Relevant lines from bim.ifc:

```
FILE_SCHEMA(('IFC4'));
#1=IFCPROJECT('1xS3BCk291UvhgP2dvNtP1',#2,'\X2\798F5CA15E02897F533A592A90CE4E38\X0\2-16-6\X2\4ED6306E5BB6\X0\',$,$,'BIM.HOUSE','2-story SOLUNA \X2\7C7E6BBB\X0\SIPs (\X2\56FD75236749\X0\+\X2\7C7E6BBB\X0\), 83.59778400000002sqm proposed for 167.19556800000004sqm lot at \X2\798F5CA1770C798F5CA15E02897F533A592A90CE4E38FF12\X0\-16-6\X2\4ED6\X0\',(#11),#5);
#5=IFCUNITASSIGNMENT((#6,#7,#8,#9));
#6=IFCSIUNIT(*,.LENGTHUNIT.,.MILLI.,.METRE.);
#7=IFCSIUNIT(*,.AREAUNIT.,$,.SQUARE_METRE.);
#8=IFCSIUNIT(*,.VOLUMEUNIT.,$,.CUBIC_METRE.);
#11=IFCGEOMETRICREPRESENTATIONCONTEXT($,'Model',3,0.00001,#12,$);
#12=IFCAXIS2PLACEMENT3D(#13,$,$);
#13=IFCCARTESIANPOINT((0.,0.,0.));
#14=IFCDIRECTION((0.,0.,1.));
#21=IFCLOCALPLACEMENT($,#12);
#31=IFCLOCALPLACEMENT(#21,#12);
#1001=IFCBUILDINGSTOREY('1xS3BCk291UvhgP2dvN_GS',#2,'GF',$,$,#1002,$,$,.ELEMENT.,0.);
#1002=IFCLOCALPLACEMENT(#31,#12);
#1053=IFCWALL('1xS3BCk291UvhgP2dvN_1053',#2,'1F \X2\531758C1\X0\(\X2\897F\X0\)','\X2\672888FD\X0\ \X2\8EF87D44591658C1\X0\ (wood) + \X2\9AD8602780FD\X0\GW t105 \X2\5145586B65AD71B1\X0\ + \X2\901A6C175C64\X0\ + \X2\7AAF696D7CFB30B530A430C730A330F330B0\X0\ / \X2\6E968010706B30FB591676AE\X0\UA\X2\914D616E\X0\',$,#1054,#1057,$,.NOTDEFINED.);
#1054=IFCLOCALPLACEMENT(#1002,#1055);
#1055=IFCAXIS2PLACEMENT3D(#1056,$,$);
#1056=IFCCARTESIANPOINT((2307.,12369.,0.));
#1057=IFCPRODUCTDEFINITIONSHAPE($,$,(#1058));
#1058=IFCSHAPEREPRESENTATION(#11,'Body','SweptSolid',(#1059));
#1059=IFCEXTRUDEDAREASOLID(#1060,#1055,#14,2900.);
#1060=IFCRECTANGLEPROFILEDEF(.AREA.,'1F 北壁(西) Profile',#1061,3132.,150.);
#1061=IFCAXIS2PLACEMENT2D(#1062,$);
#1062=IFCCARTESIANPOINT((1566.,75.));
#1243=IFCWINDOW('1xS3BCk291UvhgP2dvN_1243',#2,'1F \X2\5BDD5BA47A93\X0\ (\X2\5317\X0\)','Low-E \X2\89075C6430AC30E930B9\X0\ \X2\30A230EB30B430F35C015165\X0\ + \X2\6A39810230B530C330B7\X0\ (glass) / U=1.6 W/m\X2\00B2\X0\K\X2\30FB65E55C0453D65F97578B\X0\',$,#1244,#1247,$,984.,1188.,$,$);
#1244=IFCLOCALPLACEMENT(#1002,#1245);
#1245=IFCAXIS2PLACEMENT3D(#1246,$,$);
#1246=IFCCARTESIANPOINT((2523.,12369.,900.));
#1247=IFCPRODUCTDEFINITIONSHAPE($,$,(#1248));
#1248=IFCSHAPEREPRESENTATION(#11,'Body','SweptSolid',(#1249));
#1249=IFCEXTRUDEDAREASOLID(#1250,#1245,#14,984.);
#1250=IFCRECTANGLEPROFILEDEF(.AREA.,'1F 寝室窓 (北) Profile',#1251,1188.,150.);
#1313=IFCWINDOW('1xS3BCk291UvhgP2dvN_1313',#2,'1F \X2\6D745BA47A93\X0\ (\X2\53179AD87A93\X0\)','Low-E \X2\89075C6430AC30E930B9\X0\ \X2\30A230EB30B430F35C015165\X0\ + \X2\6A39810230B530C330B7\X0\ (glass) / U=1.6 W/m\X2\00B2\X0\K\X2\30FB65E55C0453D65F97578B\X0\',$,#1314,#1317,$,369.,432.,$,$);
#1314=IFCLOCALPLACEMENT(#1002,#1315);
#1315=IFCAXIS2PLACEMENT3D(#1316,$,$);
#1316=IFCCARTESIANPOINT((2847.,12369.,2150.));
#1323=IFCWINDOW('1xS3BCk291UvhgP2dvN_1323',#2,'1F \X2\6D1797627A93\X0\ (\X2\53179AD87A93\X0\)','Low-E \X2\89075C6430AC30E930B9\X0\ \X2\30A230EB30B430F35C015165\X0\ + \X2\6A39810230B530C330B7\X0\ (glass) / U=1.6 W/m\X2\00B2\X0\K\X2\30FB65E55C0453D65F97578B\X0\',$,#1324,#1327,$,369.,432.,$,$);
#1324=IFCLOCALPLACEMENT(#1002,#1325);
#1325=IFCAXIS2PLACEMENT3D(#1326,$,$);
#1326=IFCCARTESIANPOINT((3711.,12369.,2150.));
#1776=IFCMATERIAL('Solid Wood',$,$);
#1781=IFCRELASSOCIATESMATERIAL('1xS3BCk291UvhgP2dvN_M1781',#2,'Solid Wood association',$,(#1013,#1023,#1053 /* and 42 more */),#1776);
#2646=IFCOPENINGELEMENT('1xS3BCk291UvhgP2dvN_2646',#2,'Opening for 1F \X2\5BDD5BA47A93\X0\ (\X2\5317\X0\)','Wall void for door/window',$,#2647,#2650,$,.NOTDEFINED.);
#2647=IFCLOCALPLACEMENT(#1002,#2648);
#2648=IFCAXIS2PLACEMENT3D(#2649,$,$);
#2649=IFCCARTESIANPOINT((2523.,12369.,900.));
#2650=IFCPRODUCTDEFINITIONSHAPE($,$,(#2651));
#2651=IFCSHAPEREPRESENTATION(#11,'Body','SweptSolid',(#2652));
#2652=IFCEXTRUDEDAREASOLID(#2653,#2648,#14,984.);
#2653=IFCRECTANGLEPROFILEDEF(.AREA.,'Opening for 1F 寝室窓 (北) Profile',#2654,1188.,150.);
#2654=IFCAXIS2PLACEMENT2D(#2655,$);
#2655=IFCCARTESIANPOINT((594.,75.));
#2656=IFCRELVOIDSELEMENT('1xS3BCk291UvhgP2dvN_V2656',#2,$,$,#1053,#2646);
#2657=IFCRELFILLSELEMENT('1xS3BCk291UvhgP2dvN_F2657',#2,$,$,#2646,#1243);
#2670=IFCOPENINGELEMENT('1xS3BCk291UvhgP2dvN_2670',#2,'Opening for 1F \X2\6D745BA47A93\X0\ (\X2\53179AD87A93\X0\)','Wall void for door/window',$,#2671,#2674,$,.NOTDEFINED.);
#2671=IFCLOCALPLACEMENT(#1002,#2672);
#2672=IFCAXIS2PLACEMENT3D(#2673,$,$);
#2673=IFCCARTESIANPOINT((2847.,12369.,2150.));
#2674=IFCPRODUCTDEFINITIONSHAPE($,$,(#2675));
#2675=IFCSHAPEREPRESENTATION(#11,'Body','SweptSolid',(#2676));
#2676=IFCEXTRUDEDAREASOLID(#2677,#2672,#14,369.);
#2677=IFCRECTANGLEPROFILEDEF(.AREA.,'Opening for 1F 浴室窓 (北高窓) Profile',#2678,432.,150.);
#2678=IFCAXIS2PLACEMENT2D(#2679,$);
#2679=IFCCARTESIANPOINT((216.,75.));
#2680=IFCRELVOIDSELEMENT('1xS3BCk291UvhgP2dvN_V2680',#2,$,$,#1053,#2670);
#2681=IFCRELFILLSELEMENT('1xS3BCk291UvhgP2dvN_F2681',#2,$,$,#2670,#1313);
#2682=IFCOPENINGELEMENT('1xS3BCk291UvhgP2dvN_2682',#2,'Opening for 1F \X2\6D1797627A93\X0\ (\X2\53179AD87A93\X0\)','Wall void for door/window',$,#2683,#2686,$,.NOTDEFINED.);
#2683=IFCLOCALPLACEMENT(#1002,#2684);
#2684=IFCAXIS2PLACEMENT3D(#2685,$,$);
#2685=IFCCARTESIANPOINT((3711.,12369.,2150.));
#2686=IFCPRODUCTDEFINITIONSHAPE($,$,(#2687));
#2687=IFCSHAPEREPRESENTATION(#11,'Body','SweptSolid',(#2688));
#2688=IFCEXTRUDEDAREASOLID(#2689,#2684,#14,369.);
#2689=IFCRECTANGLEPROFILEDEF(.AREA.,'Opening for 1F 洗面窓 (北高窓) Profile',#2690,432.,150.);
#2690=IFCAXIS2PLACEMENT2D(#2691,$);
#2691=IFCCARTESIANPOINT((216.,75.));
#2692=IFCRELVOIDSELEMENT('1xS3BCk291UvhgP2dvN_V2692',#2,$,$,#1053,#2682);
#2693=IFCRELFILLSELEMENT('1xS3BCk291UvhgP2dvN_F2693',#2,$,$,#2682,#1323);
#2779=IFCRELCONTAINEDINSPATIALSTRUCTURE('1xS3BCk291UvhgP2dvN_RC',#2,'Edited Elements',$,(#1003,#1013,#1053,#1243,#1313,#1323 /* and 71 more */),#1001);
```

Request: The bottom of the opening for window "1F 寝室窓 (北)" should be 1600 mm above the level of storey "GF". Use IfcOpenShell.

```python
import numpy as np
import ifcopenshell
import ifcopenshell.api.geometry
import ifcopenshell.geom
import ifcopenshell.util.element
import ifcopenshell.util.placement
import ifcopenshell.util.shape
import ifcopenshell.util.unit

model = ifcopenshell.open("bim.ifc")
unit_scale = ifcopenshell.util.unit.calculate_unit_scale(model)

window = model.by_guid("1xS3BCk291UvhgP2dvN_1243")
opening = window.FillsVoids[0].RelatingOpeningElement
storey = ifcopenshell.util.element.get_container(window, ifc_class="IfcBuildingStorey")
level = ifcopenshell.util.placement.get_local_placement(storey.ObjectPlacement)[2, 3]

# The opening's origin need not be at the sill, so measure its lowest point.
shape = ifcopenshell.geom.create_shape(ifcopenshell.geom.settings(), opening)
bottom = ifcopenshell.util.shape.get_shape_bottom_elevation(shape, shape.geometry) / unit_scale
dz = level + 1.6 / unit_scale - bottom

shift = np.array([0.0, 0.0, dz])
# The window is not placed relative to its opening, so move both.
for product in (opening, window):
    matrix = ifcopenshell.util.placement.get_local_placement(product.ObjectPlacement)
    matrix[:3, 3] += shift
    ifcopenshell.api.geometry.edit_object_placement(model, product=product, matrix=matrix, is_si=False)

print(f"moved by {dz * unit_scale:+.3f} m")

model.write("bim_edited.ifc")
```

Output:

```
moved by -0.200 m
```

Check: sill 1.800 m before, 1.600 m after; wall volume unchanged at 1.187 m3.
